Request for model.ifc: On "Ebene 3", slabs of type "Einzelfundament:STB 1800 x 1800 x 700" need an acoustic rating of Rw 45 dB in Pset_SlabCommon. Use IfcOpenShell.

First a look at what the model holds.

```python
import ifcopenshell
import ifcopenshell.util.element

model = ifcopenshell.open("model.ifc")
print(model.schema)
storey = next(s for s in model.by_type("IfcBuildingStorey") if s.Name == "Ebene 3")
slabs = [e for e in ifcopenshell.util.element.get_decomposition(storey) if e.is_a("IfcSlab")]
seen = {}
for e in slabs:
    element_type = ifcopenshell.util.element.get_type(e)
    key = (element_type.Name if element_type != e and element_type else None, ifcopenshell.util.element.get_pset(e, "Pset_SlabCommon", "AcousticRating"))
    seen[key] = seen.get(key, 0) + 1
for (name, value), count in sorted(seen.items(), key=str):
    print(count, "x", name, "|", value)
```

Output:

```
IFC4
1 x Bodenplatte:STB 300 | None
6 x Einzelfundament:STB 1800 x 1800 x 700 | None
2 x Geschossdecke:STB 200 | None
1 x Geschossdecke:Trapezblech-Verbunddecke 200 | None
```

```python
import ifcopenshell
import ifcopenshell.api.pset
import ifcopenshell.util.element

model = ifcopenshell.open("model.ifc")

storey = next(s for s in model.by_type("IfcBuildingStorey") if s.Name == "Ebene 3")
slabs = [e for e in ifcopenshell.util.element.get_decomposition(storey) if e.is_a("IfcSlab")]

count = 0
for e in slabs:
    element_type = ifcopenshell.util.element.get_type(e)
    if element_type in (None, e) or element_type.Name != "Einzelfundament:STB 1800 x 1800 x 700":
        continue
    # add_pset returns the element's existing set when there is one.
    pset = ifcopenshell.api.pset.add_pset(model, product=e, name="Pset_SlabCommon")
    ifcopenshell.api.pset.edit_pset(model, pset=pset, properties={"AcousticRating": "Rw 45 dB"})
    count += 1

print(count, "slabs updated")

model.write("model_rev.ifc")
```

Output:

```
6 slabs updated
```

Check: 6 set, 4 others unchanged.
